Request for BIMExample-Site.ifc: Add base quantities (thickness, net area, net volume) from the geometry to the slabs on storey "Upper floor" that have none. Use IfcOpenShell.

First a look at what the model holds.

```python
import ifcopenshell
import ifcopenshell.util.element
import ifcopenshell.util.unit

model = ifcopenshell.open("BIMExample-Site.ifc")
print(model.schema)
for unit_type in ("LENGTHUNIT", "AREAUNIT", "VOLUMEUNIT"):
    print(unit_type, ifcopenshell.util.unit.calculate_unit_scale(model, unit_type))
storey = next(s for s in model.by_type("IfcBuildingStorey") if s.Name == "Upper floor")
slabs = [e for e in ifcopenshell.util.element.get_decomposition(storey) if e.is_a("IfcSlab")]
for e in sorted(slabs, key=lambda e: e.id()):
    print(e.id(), e.is_a(), e.Name, list(ifcopenshell.util.element.get_psets(e, qtos_only=True)), sep=" | ")
```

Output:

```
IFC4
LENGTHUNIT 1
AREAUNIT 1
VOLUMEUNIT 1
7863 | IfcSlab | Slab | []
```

```python
import ifcopenshell
import ifcopenshell.api.pset
import ifcopenshell.geom
import ifcopenshell.util.element
import ifcopenshell.util.shape
import ifcopenshell.util.unit

model = ifcopenshell.open("BIMExample-Site.ifc")
unit_scale = ifcopenshell.util.unit.calculate_unit_scale(model)
area_scale = ifcopenshell.util.unit.calculate_unit_scale(model, "AREAUNIT")
volume_scale = ifcopenshell.util.unit.calculate_unit_scale(model, "VOLUMEUNIT")
settings = ifcopenshell.geom.settings()

storey = next(s for s in model.by_type("IfcBuildingStorey") if s.Name == "Upper floor")
slabs = [e for e in ifcopenshell.util.element.get_decomposition(storey) if e.is_a("IfcSlab")]

for e in sorted(slabs, key=lambda e: e.id()):
    if ifcopenshell.util.element.get_psets(e, qtos_only=True, should_inherit=False):
        continue
    # Geometry comes back in metres, in the element's own axes.
    shape = ifcopenshell.geom.create_shape(settings, e)
    values = {
        "Width": ifcopenshell.util.shape.get_z(shape.geometry) / unit_scale,
        "NetArea": ifcopenshell.util.shape.get_footprint_area(shape.geometry) / area_scale,
        "NetVolume": ifcopenshell.util.shape.get_volume(shape.geometry) / volume_scale,
    }
    qto = ifcopenshell.api.pset.add_qto(model, product=e, name="Qto_SlabBaseQuantities")
    ifcopenshell.api.pset.edit_qto(model, qto=qto, properties=values)
    print(e.id(), {k: round(v, 3) for k, v in values.items()})

model.write("BIMExample-Site_edited.ifc")
```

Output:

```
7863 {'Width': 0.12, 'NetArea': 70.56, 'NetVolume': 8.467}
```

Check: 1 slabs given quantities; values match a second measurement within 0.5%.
